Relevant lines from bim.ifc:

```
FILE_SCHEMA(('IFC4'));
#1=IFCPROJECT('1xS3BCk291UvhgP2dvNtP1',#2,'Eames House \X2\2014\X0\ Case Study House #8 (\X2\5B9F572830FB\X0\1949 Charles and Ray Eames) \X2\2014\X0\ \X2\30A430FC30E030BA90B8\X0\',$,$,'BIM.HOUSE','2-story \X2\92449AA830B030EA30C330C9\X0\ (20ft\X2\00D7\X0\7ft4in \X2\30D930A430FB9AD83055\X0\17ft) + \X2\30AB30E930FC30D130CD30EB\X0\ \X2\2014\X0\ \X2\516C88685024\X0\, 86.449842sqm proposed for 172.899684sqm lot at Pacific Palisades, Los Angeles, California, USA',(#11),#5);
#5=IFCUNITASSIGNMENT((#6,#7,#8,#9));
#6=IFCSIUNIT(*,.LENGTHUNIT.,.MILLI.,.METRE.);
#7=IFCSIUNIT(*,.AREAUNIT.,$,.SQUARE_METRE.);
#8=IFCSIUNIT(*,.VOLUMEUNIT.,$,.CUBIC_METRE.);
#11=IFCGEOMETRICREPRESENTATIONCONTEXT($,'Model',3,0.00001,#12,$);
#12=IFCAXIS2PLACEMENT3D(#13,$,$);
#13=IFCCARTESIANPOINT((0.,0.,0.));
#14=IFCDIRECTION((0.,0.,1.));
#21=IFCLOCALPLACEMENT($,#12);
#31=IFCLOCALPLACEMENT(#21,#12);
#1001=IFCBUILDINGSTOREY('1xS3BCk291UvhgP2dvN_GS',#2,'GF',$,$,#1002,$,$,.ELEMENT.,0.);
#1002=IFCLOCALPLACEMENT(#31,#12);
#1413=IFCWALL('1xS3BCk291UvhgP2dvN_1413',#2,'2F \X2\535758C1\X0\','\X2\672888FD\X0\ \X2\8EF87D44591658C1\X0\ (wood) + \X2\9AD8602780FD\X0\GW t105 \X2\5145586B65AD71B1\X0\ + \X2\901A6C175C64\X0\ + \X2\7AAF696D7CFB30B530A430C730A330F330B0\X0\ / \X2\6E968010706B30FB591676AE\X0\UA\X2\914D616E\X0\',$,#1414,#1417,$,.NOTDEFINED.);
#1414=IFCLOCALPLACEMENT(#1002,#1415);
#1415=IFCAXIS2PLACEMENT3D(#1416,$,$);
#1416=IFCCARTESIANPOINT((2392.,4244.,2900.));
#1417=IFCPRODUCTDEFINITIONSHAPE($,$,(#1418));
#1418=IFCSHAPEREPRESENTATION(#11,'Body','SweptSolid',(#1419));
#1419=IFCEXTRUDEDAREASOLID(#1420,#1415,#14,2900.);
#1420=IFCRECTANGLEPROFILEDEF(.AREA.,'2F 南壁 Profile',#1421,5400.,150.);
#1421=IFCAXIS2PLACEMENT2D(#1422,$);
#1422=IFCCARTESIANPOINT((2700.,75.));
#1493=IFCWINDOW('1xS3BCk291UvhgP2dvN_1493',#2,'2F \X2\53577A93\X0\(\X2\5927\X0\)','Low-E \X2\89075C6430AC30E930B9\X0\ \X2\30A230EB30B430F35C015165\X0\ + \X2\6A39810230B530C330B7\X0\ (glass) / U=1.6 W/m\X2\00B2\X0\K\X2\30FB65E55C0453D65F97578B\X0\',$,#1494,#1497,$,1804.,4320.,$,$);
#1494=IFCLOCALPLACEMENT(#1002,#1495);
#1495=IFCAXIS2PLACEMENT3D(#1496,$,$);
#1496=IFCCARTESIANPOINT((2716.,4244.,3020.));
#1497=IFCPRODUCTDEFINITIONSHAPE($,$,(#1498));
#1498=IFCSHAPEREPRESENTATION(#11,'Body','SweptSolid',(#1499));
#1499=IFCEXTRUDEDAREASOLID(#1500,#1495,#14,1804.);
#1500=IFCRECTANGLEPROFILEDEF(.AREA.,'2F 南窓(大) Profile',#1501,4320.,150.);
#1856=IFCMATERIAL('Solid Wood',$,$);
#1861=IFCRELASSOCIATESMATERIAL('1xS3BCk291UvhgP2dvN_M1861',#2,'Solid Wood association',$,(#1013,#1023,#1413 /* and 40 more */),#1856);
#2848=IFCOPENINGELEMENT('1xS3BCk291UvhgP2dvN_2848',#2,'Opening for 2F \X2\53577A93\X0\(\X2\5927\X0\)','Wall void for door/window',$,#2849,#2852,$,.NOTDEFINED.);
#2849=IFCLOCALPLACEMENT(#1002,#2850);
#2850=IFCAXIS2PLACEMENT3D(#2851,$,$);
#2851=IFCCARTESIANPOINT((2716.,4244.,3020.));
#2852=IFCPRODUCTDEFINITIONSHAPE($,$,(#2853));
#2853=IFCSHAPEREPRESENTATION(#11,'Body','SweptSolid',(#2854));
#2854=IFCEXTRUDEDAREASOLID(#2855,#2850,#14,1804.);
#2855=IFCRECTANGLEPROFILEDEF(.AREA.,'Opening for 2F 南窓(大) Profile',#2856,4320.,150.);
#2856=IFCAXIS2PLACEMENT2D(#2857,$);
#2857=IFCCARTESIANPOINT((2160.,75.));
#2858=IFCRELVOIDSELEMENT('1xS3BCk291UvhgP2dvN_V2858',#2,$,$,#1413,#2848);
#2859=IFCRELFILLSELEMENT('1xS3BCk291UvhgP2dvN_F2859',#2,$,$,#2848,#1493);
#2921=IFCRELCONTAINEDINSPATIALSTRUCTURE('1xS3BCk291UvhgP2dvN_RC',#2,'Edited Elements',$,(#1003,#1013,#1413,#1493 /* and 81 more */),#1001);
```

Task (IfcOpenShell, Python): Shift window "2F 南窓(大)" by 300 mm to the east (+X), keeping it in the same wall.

```python
import ifcopenshell
import ifcopenshell.api.geometry
import ifcopenshell.util.placement
import ifcopenshell.util.unit

model = ifcopenshell.open("bim.ifc")
unit_scale = ifcopenshell.util.unit.calculate_unit_scale(model)

window = model.by_id(1493)
opening = window.FillsVoids[0].RelatingOpeningElement
wall = opening.VoidsElements[0].RelatingBuildingElement

wall_matrix = ifcopenshell.util.placement.get_local_placement(wall.ObjectPlacement)
shift = wall_matrix[:3, 0] * 0.3 / unit_scale
before = ifcopenshell.util.placement.get_local_placement(window.ObjectPlacement)[:3, 3].copy()

# The window is not placed relative to its opening, so move both.
for product in (opening, window):
    matrix = ifcopenshell.util.placement.get_local_placement(product.ObjectPlacement)
    matrix[:3, 3] += shift
    ifcopenshell.api.geometry.edit_object_placement(model, product=product, matrix=matrix, is_si=False)

after = ifcopenshell.util.placement.get_local_placement(window.ObjectPlacement)[:3, 3]
print("window moved by", (after - before).round(3) + 0.0)

model.write("bim_v2.ifc")
```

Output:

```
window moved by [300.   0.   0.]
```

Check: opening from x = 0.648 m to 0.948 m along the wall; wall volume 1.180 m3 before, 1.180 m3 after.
